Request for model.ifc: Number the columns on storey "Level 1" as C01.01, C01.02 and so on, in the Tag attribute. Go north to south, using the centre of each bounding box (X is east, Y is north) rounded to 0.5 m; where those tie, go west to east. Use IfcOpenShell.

First a look at what the model holds.

```python
import ifcopenshell
import ifcopenshell.util.element
import ifcopenshell.util.placement

model = ifcopenshell.open("model.ifc")
print(model.schema)
storey = next(s for s in model.by_type("IfcBuildingStorey") if s.Name == "Level 1")
columns = [e for e in ifcopenshell.util.element.get_decomposition(storey) if e.is_a("IfcColumn")]
for e in sorted(columns, key=lambda e: e.id()):
    origin = ifcopenshell.util.placement.get_local_placement(e.ObjectPlacement)[:3, 3]
    print(e.id(), e.Tag, e.Name, origin.round(2) + 0.0, sep=" | ")
```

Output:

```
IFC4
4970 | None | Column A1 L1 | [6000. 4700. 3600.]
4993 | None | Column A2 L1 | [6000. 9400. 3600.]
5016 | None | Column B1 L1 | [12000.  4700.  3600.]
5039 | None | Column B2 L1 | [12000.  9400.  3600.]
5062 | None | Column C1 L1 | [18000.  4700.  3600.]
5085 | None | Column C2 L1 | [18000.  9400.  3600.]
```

```python
import ifcopenshell
import ifcopenshell.geom
import ifcopenshell.util.element
import ifcopenshell.util.shape

model = ifcopenshell.open("model.ifc")
settings = ifcopenshell.geom.settings()
settings.set("use-world-coords", True)


def centre(element):
    shape = ifcopenshell.geom.create_shape(settings, element)
    return ifcopenshell.util.shape.get_bbox_centroid(shape.geometry)


storey = next(s for s in model.by_type("IfcBuildingStorey") if s.Name == "Level 1")
columns = [e for e in ifcopenshell.util.element.get_decomposition(storey) if e.is_a("IfcColumn")]

# Insertion points can sit at a corner or the storey origin, so sort by the geometry (in metres).
centres = {e: centre(e) for e in columns}
columns.sort(key=lambda e: (-round(centres[e][1] / 0.5), centres[e][0]))

for i, e in enumerate(columns, start=1):
    number = f"C01.{i:02d}"
    e.Tag = number
    print(e.id(), number)

model.write("model_edited.ifc")
```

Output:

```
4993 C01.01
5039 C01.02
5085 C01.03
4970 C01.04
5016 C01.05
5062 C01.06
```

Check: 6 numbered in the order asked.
